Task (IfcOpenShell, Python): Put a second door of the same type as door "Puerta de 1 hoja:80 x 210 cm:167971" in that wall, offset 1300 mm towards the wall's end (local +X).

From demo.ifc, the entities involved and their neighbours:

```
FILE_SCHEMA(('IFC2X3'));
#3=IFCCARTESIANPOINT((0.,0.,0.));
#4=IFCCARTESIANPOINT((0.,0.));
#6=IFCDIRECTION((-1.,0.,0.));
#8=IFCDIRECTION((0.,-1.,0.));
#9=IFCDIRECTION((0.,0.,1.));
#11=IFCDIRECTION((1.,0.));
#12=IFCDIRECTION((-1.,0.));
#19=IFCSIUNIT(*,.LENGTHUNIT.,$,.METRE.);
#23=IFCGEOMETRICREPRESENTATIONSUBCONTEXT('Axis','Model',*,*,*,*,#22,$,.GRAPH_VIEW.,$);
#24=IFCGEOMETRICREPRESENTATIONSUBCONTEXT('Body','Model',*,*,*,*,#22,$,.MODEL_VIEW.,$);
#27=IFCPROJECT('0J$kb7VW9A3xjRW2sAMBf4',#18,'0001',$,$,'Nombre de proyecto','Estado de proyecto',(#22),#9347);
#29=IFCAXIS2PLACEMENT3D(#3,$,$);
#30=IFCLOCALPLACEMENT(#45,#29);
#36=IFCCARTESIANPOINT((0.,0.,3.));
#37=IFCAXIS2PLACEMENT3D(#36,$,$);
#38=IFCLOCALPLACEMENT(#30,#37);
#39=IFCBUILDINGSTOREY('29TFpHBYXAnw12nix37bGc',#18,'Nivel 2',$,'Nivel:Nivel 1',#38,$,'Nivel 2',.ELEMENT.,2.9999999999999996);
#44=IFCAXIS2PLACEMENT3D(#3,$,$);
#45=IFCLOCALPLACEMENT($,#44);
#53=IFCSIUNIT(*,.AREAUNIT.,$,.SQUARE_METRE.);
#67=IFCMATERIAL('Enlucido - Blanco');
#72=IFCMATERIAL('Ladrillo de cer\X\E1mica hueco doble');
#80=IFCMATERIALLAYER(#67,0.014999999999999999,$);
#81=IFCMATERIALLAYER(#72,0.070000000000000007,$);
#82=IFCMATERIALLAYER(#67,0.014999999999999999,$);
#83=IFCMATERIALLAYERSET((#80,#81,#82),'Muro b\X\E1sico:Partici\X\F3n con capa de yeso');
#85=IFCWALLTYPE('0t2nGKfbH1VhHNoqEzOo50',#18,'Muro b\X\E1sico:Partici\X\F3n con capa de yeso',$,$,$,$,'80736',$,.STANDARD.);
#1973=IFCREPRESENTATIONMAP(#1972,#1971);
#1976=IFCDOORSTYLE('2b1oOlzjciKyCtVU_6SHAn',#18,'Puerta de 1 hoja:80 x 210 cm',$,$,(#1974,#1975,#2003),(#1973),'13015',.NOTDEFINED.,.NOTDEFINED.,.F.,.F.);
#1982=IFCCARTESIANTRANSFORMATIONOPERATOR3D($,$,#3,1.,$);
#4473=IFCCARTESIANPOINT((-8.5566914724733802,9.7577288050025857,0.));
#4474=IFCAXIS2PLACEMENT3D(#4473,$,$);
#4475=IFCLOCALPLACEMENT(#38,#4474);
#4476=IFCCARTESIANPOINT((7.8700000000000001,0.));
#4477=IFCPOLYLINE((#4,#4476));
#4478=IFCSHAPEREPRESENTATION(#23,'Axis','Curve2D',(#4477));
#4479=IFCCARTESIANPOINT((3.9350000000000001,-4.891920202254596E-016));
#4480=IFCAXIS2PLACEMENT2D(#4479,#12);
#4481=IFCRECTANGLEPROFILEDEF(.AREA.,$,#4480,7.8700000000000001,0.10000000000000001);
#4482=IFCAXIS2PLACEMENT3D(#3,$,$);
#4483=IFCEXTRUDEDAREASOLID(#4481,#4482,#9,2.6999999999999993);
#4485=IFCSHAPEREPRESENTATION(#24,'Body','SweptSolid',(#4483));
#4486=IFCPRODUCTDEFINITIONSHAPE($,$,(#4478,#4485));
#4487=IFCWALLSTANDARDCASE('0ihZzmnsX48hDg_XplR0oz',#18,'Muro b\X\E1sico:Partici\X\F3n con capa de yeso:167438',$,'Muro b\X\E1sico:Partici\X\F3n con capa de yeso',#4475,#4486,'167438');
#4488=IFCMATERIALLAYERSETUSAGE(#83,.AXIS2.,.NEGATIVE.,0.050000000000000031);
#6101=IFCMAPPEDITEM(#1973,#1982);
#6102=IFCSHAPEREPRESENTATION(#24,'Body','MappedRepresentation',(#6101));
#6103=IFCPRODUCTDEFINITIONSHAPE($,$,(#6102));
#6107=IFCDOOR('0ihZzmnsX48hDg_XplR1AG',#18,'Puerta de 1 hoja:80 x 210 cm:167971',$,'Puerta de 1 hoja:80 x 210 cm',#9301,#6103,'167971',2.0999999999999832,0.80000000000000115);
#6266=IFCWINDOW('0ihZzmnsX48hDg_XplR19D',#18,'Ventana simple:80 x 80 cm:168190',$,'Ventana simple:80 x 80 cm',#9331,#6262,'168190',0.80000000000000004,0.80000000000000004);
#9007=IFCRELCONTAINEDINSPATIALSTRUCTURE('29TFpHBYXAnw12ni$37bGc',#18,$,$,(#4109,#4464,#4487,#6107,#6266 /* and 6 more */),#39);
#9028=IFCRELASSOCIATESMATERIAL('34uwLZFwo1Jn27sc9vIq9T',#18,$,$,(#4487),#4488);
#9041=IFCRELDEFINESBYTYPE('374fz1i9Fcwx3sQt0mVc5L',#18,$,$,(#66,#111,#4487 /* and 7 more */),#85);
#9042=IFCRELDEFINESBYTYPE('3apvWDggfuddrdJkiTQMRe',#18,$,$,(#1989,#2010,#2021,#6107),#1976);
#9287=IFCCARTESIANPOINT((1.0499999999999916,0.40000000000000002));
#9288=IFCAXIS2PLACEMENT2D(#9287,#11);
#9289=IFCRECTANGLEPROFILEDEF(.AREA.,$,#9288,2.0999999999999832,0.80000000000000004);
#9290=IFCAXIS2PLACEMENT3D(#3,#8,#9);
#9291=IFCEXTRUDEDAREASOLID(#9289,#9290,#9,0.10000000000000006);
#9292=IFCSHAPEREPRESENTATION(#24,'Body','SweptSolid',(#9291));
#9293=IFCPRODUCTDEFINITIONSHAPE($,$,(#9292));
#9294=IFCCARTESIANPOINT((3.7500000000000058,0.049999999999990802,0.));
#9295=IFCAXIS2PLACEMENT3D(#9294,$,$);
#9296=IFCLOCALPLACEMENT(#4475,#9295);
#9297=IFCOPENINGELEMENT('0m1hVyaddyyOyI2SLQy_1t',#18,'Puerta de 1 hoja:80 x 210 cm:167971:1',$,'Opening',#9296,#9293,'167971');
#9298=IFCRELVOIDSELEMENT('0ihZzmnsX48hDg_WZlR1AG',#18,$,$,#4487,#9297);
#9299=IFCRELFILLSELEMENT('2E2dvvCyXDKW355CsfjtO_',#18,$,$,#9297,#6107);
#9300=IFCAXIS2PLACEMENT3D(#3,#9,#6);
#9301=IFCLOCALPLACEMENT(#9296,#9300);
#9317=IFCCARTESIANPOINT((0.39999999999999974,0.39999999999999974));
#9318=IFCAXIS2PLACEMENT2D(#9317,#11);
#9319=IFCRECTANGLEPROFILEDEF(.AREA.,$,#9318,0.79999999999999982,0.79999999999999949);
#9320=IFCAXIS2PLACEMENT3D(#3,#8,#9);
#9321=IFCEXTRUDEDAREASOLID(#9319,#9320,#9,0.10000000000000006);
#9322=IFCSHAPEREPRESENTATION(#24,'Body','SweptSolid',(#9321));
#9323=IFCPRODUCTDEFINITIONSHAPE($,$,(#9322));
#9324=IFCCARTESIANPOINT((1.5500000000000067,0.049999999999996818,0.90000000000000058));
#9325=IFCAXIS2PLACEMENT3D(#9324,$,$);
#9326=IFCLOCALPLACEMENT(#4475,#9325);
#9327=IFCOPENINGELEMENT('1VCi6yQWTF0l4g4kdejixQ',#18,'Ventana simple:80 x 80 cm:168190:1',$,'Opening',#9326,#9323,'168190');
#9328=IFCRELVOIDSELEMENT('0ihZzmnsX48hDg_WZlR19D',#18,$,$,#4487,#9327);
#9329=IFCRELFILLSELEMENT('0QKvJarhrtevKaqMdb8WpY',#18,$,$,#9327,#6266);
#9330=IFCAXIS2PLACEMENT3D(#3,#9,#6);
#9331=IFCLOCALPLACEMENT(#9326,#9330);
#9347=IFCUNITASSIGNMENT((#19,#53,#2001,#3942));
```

```python
import ifcopenshell
import ifcopenshell.api.feature
import ifcopenshell.api.geometry
import ifcopenshell.api.root
import ifcopenshell.geom
import ifcopenshell.util.element
import ifcopenshell.util.placement
import ifcopenshell.util.shape
import ifcopenshell.util.unit

model = ifcopenshell.open("demo.ifc")
unit_scale = ifcopenshell.util.unit.calculate_unit_scale(model)
settings = ifcopenshell.geom.settings()


def volume(element):
    """Net volume in cubic metres, openings subtracted."""
    shape = ifcopenshell.geom.create_shape(settings, element)
    return ifcopenshell.util.shape.get_volume(shape.geometry)


def reuse_history(source, copy):
    """copy_class also copies each property set's owner history, people and application; keep the originals."""
    for rel in copy.IsDefinedBy:
        if rel.is_a("IfcRelDefinesByProperties") and (history := rel.RelatingPropertyDefinition.OwnerHistory):
            rel.RelatingPropertyDefinition.OwnerHistory = source.OwnerHistory
            ifcopenshell.util.element.remove_deep2(model, history)


door = model.by_id(6107)
opening = door.FillsVoids[0].RelatingOpeningElement
wall = opening.VoidsElements[0].RelatingBuildingElement
before = volume(wall)
shift = ifcopenshell.util.placement.get_local_placement(wall.ObjectPlacement)[:3, 0] * 1.3 / unit_scale

# copy_class copies the void relationship, type, container and properties, but no geometry.
new_opening = ifcopenshell.api.root.copy_class(model, product=opening)
new_opening.Representation = ifcopenshell.util.element.copy_deep(
    model, opening.Representation, exclude=["IfcGeometricRepresentationContext", "IfcRepresentationMap"]
)
new_opening.Name = "Puerta de 1 hoja:80 x 210 cm"
new_opening.Tag = None
new_door = ifcopenshell.api.root.copy_class(model, product=door)
new_door.Representation = ifcopenshell.util.element.copy_deep(
    model, door.Representation, exclude=["IfcGeometricRepresentationContext", "IfcRepresentationMap"]
)
new_door.Name = "Puerta de 1 hoja:80 x 210 cm"
new_door.Tag = None
reuse_history(door, new_door)
fills = ifcopenshell.api.feature.add_filling(model, opening=new_opening, element=new_door)
fills.OwnerHistory = new_door.OwnerHistory  # required in IFC2X3

for old, new in ((opening, new_opening), (door, new_door)):
    matrix = ifcopenshell.util.placement.get_local_placement(old.ObjectPlacement)
    matrix[:3, 3] += shift
    ifcopenshell.api.geometry.edit_object_placement(model, product=new, matrix=matrix, is_si=False)

after = volume(wall)

print(f"wall volume {before:.3f} -> {after:.3f} m3")

model.write("demo_edited.ifc")
```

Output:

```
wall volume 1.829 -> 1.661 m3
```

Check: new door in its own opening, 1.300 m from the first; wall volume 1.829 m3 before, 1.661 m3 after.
